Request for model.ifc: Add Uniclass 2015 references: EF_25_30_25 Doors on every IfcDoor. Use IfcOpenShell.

First a look at what the model holds.

```python
import ifcopenshell

model = ifcopenshell.open("model.ifc")
print(model.schema)
print("classifications:", [c.Name for c in model.by_type("IfcClassification")])
for ifc_class in ("IfcDoor", "IfcRoof", "IfcStair", "IfcWall", "IfcWindow"):
    print(ifc_class, len(model.by_type(ifc_class)))
```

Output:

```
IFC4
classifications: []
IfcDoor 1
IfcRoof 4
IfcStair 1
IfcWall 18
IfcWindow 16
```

```python
import ifcopenshell
import ifcopenshell.api.classification

model = ifcopenshell.open("model.ifc")

system = ifcopenshell.api.classification.add_classification(model, classification="Uniclass 2015")

codes = {
    "IfcDoor": ("EF_25_30_25", "Doors"),
}
for ifc_class, (code, name) in codes.items():
    products = model.by_type(ifc_class)
    ifcopenshell.api.classification.add_reference(
        model, products=products, classification=system, identification=code, name=name
    )
    print(code, len(products))

model.write("model_edited.ifc")
```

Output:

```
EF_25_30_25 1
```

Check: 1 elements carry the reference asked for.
